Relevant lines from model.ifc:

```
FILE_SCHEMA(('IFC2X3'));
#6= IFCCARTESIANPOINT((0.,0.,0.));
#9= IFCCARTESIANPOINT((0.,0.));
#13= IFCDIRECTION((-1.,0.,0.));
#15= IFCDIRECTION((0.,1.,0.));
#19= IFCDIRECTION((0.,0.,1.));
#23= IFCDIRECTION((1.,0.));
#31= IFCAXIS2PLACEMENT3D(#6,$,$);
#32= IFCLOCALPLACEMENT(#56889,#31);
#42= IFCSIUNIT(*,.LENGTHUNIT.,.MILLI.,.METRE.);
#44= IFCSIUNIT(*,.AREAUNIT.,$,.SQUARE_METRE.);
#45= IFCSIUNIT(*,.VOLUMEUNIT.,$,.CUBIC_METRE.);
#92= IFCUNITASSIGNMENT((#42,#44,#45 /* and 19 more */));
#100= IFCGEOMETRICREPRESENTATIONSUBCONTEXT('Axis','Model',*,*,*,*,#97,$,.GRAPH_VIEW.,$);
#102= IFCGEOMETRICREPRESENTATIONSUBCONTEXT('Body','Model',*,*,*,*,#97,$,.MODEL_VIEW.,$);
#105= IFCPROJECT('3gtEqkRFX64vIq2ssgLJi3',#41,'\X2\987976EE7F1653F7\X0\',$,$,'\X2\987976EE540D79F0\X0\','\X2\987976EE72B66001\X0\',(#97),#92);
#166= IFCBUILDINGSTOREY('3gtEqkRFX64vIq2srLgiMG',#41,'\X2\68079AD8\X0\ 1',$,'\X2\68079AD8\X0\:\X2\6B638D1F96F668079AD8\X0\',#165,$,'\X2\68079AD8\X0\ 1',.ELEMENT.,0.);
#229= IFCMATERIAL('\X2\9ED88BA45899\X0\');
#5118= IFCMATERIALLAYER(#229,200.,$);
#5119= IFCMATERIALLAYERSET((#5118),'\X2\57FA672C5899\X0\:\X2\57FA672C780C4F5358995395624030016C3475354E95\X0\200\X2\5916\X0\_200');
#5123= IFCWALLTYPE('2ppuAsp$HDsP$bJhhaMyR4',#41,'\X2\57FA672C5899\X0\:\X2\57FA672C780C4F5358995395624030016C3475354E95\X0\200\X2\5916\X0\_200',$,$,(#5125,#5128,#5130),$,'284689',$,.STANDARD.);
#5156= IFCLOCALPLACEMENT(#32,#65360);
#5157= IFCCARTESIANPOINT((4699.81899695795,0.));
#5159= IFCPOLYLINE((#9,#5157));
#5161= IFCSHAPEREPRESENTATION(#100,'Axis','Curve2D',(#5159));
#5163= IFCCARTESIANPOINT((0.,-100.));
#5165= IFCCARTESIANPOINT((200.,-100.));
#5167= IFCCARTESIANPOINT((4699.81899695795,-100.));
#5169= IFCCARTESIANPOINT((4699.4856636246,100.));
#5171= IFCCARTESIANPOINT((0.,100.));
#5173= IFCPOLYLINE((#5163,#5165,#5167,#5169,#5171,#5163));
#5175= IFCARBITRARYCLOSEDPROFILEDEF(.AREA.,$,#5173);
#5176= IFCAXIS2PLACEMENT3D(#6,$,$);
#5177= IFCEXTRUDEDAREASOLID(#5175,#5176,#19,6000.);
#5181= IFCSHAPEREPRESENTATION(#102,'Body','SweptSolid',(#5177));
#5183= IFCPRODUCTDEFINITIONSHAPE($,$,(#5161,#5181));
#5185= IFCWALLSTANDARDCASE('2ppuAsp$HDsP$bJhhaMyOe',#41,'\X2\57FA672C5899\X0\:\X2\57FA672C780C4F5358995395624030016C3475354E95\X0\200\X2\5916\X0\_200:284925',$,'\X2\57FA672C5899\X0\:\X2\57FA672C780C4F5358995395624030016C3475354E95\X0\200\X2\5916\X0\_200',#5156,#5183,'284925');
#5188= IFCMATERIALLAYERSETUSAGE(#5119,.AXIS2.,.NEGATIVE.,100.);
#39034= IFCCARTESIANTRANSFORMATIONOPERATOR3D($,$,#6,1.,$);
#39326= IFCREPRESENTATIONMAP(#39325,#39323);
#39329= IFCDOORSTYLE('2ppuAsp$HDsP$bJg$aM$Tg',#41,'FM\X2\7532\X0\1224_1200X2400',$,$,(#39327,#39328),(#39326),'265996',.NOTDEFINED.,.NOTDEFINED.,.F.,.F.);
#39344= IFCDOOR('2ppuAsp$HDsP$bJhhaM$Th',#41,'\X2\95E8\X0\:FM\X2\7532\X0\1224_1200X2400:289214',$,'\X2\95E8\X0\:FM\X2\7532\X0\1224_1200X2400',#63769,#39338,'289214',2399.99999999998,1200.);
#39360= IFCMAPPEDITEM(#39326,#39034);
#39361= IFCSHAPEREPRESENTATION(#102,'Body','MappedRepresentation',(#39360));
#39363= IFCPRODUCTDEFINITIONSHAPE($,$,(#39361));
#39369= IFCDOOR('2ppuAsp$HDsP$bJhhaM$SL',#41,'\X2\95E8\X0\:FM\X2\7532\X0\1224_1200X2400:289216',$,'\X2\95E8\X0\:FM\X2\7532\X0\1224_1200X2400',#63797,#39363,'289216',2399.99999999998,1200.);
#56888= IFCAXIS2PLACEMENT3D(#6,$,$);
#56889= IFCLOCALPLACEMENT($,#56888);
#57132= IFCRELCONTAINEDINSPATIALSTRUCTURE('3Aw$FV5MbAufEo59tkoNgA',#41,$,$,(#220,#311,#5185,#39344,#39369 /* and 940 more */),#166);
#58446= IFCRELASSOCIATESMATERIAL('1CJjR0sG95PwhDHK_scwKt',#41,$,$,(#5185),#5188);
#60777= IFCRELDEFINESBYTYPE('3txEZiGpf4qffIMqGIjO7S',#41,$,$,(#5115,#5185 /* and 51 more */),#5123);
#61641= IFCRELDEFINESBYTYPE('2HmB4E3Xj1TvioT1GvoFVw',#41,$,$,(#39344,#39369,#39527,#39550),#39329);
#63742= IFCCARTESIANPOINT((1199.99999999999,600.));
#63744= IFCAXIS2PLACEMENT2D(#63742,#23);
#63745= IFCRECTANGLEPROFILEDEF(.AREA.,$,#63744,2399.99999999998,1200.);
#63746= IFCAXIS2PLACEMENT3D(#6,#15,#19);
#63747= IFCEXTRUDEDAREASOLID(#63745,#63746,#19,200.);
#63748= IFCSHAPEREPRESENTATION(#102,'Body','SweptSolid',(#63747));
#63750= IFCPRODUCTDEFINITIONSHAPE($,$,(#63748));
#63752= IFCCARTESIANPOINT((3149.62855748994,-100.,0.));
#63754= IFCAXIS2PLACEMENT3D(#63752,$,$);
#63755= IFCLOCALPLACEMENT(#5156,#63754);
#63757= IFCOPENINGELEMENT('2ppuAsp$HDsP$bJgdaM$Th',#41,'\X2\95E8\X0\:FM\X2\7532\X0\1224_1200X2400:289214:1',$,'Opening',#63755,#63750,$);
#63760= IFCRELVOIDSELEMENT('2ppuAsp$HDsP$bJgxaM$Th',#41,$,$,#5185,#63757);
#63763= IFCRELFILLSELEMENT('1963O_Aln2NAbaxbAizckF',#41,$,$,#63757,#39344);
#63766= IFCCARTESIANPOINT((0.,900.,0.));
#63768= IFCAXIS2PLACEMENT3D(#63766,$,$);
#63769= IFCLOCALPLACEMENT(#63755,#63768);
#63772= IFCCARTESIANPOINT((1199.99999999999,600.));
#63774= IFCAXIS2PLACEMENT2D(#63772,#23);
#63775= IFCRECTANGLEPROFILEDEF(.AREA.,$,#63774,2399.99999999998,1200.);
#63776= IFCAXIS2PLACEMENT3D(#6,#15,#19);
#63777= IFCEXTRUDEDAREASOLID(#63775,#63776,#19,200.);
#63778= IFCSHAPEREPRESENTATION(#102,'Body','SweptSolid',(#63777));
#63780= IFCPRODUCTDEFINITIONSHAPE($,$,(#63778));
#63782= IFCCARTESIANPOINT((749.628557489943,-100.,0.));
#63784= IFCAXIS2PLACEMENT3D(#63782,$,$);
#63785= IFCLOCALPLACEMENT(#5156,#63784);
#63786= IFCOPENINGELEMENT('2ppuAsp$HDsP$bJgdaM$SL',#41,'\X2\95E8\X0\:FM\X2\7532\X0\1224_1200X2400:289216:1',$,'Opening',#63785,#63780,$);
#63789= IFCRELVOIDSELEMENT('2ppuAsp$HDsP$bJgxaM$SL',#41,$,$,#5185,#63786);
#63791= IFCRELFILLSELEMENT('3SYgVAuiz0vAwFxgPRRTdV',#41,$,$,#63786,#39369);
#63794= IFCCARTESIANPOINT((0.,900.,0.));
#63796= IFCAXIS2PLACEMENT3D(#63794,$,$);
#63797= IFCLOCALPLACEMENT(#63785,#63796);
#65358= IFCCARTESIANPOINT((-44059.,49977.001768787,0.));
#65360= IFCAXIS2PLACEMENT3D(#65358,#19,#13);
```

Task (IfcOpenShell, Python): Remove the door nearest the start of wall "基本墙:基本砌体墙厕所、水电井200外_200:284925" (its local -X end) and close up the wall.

```python
import ifcopenshell
import ifcopenshell.api.feature
import ifcopenshell.api.root
import ifcopenshell.geom
import ifcopenshell.util.shape

model = ifcopenshell.open("model.ifc")
settings = ifcopenshell.geom.settings()


def volume(element):
    """Net volume in cubic metres, openings subtracted."""
    shape = ifcopenshell.geom.create_shape(settings, element)
    return ifcopenshell.util.shape.get_volume(shape.geometry)


door = model.by_guid("2ppuAsp$HDsP$bJhhaM$SL")
opening = door.FillsVoids[0].RelatingOpeningElement
wall = opening.VoidsElements[0].RelatingBuildingElement
before = volume(wall)

ifcopenshell.api.root.remove_product(model, product=door)
ifcopenshell.api.feature.remove_feature(model, feature=opening)

after = volume(wall)

print(f"wall volume {before:.3f} -> {after:.3f} m3")

model.write("model-out.ifc")
```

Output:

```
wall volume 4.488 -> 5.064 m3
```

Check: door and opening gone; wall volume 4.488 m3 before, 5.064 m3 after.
